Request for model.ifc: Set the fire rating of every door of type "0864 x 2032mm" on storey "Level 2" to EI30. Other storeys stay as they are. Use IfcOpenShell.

First a look at what the model holds.

```python
import ifcopenshell
import ifcopenshell.util.element

model = ifcopenshell.open("model.ifc")
print(model.schema)
storey = next(s for s in model.by_type("IfcBuildingStorey") if s.Name == "Level 2")
doors = [e for e in ifcopenshell.util.element.get_decomposition(storey) if e.is_a("IfcDoor")]
seen = {}
for e in doors:
    element_type = ifcopenshell.util.element.get_type(e)
    key = (element_type.Name if element_type != e and element_type else None, ifcopenshell.util.element.get_pset(e, "Pset_DoorCommon", "FireRating"))
    seen[key] = seen.get(key, 0) + 1
for (name, value), count in sorted(seen.items(), key=str):
    print(count, "x", name, "|", value)
```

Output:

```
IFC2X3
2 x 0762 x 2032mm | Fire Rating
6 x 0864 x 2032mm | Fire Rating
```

```python
import ifcopenshell
import ifcopenshell.api.pset
import ifcopenshell.util.element

model = ifcopenshell.open("model.ifc")

storey = next(s for s in model.by_type("IfcBuildingStorey") if s.Name == "Level 2")
doors = [e for e in ifcopenshell.util.element.get_decomposition(storey) if e.is_a("IfcDoor")]

count = 0
for e in doors:
    element_type = ifcopenshell.util.element.get_type(e)
    if element_type in (None, e) or element_type.Name != "0864 x 2032mm":
        continue
    # add_pset returns the element's existing set when there is one.
    pset = ifcopenshell.api.pset.add_pset(model, product=e, name="Pset_DoorCommon")
    ifcopenshell.api.pset.edit_pset(model, pset=pset, properties={"FireRating": "EI30"})
    count += 1

print(count, "doors updated")

model.write("model_updated.ifc")
```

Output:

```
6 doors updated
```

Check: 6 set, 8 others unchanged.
